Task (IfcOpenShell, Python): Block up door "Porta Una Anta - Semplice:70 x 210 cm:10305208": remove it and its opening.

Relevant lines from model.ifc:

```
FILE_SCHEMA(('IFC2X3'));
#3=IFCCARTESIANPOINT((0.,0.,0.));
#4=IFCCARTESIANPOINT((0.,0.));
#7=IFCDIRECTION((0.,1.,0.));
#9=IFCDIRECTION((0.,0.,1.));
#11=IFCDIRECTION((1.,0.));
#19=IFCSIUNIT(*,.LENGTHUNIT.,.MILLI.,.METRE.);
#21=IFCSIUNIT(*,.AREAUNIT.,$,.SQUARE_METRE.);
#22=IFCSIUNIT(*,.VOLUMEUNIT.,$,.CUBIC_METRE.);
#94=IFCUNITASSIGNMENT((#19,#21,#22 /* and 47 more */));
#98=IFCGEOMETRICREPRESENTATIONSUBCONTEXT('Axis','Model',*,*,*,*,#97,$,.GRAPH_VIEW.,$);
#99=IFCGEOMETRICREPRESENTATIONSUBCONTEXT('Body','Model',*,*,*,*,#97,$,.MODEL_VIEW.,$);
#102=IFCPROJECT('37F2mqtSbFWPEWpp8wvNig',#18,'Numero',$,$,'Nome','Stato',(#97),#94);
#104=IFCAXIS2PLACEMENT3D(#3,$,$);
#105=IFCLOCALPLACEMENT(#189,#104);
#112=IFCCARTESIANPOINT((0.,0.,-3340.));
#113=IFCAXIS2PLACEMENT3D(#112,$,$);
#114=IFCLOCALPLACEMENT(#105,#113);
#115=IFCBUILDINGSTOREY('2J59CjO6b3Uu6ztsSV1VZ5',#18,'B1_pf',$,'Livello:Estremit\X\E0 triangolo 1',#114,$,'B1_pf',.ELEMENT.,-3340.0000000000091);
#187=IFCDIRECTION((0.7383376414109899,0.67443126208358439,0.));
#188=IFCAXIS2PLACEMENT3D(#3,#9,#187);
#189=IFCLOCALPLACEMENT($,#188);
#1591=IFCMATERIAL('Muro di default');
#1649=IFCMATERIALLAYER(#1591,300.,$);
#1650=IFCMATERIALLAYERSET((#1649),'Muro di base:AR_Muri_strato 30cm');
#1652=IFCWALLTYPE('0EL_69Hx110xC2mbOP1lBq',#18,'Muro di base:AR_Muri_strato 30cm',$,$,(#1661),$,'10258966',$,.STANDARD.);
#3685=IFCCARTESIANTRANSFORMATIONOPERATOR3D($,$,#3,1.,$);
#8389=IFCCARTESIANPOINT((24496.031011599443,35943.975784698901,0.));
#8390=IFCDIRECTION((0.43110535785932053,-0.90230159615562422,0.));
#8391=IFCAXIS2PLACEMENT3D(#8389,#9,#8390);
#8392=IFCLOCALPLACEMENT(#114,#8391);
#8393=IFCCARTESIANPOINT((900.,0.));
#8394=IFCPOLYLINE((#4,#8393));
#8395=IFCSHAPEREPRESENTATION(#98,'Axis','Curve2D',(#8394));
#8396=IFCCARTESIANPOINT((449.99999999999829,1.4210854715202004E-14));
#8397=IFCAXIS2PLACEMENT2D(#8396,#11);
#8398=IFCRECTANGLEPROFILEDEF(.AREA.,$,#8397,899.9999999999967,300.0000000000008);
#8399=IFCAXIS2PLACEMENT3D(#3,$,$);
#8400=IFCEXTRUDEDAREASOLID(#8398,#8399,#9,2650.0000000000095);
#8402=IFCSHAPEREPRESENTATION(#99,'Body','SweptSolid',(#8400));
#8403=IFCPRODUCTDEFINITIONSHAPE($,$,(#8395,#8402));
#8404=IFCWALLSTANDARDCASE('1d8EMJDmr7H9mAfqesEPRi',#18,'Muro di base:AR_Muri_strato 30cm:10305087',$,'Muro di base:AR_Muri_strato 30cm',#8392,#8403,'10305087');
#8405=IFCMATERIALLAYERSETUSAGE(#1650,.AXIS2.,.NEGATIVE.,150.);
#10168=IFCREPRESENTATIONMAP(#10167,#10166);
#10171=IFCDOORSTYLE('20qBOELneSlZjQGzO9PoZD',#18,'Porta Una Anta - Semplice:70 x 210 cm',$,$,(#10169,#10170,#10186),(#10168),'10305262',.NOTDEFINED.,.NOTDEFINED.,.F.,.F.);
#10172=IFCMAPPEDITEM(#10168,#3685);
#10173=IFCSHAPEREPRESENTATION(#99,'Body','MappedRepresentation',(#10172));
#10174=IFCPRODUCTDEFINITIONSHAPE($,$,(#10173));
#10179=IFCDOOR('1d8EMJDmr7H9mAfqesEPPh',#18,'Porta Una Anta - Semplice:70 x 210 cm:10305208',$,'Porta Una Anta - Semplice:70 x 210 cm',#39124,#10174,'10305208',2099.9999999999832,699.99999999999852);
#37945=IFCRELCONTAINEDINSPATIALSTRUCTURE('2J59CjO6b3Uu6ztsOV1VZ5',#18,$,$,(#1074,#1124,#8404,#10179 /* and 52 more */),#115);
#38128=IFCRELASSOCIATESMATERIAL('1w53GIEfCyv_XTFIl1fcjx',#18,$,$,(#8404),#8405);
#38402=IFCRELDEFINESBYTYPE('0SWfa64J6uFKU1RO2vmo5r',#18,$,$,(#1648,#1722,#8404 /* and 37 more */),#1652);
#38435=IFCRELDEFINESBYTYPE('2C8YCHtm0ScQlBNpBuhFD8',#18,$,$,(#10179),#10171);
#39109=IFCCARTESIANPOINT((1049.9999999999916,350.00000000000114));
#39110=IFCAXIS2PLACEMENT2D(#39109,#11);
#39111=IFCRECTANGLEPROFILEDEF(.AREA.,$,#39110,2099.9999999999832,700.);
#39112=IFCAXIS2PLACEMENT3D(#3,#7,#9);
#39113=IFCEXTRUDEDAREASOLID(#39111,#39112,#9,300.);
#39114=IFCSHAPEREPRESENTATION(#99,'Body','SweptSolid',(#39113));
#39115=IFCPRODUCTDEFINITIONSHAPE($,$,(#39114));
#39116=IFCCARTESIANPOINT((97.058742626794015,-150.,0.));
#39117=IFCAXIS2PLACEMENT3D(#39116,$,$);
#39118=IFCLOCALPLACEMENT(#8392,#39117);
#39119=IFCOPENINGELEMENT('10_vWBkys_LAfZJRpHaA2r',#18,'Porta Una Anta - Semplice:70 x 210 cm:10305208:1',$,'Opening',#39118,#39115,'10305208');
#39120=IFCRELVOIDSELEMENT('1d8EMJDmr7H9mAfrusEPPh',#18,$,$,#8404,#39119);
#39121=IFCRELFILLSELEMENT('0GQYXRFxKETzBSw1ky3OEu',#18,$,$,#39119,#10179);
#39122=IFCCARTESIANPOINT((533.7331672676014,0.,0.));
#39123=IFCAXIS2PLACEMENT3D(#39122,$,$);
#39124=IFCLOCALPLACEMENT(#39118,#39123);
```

```python
import ifcopenshell
import ifcopenshell.api.feature
import ifcopenshell.api.root
import ifcopenshell.geom
import ifcopenshell.util.shape

model = ifcopenshell.open("model.ifc")
settings = ifcopenshell.geom.settings()


def volume(element):
    """Net volume in cubic metres, openings subtracted."""
    shape = ifcopenshell.geom.create_shape(settings, element)
    return ifcopenshell.util.shape.get_volume(shape.geometry)


door = model.by_guid("1d8EMJDmr7H9mAfqesEPPh")
opening = door.FillsVoids[0].RelatingOpeningElement
wall = opening.VoidsElements[0].RelatingBuildingElement
before = volume(wall)

ifcopenshell.api.root.remove_product(model, product=door)
ifcopenshell.api.feature.remove_feature(model, feature=opening)

after = volume(wall)

print(f"wall volume {before:.3f} -> {after:.3f} m3")

model.write("model_updated.ifc")
```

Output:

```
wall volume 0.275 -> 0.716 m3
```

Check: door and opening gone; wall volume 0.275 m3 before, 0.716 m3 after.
